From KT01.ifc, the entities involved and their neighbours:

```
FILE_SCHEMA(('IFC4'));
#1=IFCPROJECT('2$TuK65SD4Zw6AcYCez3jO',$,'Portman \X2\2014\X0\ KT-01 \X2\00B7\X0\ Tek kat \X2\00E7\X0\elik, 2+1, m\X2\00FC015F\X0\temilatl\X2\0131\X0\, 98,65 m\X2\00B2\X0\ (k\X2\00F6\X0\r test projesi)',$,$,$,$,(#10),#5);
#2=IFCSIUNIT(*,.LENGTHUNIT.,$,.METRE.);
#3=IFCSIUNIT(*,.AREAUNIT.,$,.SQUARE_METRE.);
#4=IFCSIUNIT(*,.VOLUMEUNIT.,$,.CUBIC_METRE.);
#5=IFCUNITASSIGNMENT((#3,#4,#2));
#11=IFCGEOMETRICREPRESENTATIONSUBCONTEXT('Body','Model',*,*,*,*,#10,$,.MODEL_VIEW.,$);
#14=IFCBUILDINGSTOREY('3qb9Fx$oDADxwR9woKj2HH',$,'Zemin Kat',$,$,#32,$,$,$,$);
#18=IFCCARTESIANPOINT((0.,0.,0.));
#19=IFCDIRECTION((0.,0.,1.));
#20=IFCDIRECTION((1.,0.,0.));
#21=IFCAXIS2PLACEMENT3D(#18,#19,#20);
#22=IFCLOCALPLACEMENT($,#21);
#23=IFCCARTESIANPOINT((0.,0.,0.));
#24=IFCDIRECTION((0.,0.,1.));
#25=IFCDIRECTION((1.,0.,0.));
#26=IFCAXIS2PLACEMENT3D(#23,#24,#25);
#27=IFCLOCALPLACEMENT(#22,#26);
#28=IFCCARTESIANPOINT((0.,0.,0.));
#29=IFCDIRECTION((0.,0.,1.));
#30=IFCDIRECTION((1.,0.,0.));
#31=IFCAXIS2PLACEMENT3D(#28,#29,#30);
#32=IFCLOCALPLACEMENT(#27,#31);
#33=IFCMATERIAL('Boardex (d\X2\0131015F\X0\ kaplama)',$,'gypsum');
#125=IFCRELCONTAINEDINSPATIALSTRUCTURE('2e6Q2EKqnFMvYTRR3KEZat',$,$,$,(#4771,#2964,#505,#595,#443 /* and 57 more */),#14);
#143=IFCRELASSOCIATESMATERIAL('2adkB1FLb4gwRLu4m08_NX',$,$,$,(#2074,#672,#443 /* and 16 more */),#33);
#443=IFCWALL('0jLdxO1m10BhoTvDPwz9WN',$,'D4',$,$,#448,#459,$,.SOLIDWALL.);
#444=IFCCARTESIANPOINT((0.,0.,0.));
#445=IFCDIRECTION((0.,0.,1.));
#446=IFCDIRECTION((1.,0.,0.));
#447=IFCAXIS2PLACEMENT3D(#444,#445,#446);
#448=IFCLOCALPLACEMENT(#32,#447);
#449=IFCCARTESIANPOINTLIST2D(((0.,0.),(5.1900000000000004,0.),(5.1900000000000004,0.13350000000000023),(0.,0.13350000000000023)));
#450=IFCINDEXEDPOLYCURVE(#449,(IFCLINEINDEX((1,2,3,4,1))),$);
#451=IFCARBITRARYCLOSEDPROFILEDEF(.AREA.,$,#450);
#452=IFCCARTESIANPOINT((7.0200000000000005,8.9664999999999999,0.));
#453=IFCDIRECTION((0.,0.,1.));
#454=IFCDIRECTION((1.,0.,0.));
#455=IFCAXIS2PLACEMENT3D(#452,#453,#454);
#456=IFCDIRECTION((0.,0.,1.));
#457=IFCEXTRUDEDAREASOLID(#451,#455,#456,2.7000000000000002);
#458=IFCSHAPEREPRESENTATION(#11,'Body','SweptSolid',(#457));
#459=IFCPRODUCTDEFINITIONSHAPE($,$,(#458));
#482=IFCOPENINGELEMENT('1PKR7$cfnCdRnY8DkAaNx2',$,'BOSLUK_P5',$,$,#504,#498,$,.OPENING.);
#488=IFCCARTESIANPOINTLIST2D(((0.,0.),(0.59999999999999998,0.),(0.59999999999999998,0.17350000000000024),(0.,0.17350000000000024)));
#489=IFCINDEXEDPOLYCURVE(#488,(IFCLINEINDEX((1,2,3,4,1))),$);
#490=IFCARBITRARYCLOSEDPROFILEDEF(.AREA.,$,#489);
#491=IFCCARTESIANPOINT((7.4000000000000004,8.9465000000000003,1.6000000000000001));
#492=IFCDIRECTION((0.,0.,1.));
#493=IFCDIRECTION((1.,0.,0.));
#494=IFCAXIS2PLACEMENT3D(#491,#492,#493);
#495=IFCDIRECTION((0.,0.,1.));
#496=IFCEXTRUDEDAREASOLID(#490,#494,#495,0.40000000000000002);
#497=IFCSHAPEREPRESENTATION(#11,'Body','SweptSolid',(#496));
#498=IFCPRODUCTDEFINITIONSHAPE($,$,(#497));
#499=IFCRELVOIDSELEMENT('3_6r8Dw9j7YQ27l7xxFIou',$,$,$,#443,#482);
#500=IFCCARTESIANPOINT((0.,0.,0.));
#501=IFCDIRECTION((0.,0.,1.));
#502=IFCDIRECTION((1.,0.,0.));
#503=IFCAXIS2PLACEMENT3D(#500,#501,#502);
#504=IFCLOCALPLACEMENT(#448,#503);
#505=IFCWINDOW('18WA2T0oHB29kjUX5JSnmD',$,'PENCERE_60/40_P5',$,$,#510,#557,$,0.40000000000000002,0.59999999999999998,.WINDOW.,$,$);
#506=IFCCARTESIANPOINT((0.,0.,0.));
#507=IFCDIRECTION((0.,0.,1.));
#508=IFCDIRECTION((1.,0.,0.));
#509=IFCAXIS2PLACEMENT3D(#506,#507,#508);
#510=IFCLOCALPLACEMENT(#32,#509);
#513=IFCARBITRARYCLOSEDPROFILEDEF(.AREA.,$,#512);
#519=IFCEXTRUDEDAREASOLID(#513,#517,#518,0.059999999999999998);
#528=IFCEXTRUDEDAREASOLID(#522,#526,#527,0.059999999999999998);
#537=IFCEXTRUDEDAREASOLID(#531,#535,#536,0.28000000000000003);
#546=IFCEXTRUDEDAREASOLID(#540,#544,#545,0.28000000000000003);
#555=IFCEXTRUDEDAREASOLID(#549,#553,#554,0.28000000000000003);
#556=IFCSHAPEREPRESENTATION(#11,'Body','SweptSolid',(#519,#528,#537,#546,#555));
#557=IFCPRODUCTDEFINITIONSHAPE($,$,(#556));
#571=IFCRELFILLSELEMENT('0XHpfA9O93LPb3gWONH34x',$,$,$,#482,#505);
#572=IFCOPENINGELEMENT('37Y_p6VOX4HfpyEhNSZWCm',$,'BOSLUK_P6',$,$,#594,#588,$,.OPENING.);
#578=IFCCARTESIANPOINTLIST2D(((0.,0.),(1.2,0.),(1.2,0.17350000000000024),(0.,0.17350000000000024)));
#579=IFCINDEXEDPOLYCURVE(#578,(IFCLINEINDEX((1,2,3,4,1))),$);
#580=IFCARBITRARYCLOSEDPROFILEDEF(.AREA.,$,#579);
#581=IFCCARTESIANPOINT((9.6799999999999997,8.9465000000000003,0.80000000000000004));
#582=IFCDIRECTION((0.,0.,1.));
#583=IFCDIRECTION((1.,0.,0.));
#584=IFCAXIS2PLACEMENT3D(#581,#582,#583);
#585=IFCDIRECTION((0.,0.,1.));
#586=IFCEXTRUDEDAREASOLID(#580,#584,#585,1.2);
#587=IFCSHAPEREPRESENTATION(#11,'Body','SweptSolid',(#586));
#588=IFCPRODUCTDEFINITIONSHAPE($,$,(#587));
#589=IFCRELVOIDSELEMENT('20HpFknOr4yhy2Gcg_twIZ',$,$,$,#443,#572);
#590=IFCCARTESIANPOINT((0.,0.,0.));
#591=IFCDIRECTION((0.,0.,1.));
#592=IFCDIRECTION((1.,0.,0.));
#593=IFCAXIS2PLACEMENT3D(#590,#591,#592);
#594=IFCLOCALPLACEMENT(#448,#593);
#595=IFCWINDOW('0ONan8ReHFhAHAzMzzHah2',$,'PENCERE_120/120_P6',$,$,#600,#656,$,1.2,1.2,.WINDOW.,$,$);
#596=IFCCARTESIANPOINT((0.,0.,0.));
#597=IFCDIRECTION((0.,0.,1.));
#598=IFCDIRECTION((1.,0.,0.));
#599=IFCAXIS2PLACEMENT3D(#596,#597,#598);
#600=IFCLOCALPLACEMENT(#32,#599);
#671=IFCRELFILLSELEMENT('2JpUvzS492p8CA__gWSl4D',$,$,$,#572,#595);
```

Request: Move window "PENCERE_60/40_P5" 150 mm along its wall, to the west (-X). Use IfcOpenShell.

```python
import ifcopenshell
import ifcopenshell.api.geometry
import ifcopenshell.util.placement
import ifcopenshell.util.unit

model = ifcopenshell.open("KT01.ifc")
unit_scale = ifcopenshell.util.unit.calculate_unit_scale(model)

window = model.by_id(505)
opening = window.FillsVoids[0].RelatingOpeningElement
wall = opening.VoidsElements[0].RelatingBuildingElement

wall_matrix = ifcopenshell.util.placement.get_local_placement(wall.ObjectPlacement)
shift = wall_matrix[:3, 0] * -0.15 / unit_scale
before = ifcopenshell.util.placement.get_local_placement(window.ObjectPlacement)[:3, 3].copy()

# The window is not placed relative to its opening, so move both.
for product in (opening, window):
    matrix = ifcopenshell.util.placement.get_local_placement(product.ObjectPlacement)
    matrix[:3, 3] += shift
    ifcopenshell.api.geometry.edit_object_placement(model, product=product, matrix=matrix, is_si=False)

after = ifcopenshell.util.placement.get_local_placement(window.ObjectPlacement)[:3, 3]
print("window moved by", (after - before).round(3) + 0.0)

model.write("KT01_v2.ifc")
```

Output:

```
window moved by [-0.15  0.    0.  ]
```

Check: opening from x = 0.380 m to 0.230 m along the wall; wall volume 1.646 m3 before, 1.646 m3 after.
